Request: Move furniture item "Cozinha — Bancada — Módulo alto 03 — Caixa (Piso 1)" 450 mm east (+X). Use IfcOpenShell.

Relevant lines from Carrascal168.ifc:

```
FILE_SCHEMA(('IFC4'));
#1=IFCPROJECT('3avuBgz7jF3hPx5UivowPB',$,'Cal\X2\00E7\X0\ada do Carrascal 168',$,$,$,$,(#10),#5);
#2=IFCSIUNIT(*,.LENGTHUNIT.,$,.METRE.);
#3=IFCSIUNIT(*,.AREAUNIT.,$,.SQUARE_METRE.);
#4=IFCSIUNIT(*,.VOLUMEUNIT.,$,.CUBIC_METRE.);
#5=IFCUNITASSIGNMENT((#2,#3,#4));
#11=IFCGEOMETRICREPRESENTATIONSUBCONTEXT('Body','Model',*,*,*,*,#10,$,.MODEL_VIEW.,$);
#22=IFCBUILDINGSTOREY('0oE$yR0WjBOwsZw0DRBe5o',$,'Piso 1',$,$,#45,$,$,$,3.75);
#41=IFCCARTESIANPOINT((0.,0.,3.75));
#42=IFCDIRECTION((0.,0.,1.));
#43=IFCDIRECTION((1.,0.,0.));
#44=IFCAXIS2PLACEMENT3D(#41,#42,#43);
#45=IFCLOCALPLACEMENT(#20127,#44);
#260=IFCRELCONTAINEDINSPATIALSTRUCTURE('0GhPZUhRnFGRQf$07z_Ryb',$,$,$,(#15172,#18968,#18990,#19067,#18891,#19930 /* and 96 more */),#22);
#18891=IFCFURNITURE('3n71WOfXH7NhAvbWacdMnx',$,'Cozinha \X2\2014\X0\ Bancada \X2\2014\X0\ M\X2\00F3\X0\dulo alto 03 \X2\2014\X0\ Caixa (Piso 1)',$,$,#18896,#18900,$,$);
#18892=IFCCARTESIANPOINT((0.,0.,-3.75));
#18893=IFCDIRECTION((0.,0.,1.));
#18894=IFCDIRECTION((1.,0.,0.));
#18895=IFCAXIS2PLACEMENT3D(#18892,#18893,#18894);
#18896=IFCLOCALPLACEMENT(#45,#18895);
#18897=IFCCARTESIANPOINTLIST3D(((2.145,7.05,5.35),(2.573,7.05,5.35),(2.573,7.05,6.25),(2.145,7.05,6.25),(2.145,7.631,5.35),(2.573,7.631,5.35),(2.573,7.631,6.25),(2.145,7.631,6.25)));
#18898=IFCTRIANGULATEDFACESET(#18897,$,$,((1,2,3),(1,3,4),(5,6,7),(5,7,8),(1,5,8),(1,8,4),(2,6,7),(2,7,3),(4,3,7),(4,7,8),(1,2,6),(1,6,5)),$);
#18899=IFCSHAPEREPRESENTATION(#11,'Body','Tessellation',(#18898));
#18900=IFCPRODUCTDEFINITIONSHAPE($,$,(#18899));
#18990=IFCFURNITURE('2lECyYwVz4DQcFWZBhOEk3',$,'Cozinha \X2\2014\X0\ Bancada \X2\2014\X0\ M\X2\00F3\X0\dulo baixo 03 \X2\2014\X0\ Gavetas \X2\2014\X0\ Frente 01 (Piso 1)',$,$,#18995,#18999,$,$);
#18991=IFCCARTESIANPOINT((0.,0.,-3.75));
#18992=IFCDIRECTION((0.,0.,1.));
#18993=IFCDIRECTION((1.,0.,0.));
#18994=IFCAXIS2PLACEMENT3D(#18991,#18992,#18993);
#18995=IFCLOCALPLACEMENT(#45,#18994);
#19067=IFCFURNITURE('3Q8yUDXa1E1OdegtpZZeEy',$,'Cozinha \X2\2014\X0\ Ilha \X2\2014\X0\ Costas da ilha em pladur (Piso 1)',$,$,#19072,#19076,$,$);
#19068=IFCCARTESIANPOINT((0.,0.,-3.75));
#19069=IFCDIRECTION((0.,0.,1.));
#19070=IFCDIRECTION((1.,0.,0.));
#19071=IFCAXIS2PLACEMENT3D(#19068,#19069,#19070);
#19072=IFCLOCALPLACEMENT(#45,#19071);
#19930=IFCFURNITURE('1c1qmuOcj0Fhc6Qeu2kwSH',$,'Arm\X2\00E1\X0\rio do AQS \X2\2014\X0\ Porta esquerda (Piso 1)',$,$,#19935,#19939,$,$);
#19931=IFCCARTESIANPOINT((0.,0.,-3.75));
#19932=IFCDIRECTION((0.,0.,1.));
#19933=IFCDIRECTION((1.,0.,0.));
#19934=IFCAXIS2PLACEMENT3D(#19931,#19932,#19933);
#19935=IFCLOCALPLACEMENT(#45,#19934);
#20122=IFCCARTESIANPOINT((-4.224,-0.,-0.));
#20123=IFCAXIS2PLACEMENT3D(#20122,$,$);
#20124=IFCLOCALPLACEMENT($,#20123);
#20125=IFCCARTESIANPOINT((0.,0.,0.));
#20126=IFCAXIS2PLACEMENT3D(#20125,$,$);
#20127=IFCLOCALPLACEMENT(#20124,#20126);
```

```python
import ifcopenshell
import ifcopenshell.api.geometry
import ifcopenshell.util.placement
import ifcopenshell.util.unit

model = ifcopenshell.open("Carrascal168.ifc")
unit_scale = ifcopenshell.util.unit.calculate_unit_scale(model)

item = model.by_guid("3n71WOfXH7NhAvbWacdMnx")
matrix = ifcopenshell.util.placement.get_local_placement(item.ObjectPlacement)
matrix[0, 3] += 0.45 / unit_scale
ifcopenshell.api.geometry.edit_object_placement(model, product=item, matrix=matrix, is_si=False)

print(ifcopenshell.util.placement.get_local_placement(item.ObjectPlacement).round(3) + 0.0)

model.write("Carrascal168-out.ifc")
```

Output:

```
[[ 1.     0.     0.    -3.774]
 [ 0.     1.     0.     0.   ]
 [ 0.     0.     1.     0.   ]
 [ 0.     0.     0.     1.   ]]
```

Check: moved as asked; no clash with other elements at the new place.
